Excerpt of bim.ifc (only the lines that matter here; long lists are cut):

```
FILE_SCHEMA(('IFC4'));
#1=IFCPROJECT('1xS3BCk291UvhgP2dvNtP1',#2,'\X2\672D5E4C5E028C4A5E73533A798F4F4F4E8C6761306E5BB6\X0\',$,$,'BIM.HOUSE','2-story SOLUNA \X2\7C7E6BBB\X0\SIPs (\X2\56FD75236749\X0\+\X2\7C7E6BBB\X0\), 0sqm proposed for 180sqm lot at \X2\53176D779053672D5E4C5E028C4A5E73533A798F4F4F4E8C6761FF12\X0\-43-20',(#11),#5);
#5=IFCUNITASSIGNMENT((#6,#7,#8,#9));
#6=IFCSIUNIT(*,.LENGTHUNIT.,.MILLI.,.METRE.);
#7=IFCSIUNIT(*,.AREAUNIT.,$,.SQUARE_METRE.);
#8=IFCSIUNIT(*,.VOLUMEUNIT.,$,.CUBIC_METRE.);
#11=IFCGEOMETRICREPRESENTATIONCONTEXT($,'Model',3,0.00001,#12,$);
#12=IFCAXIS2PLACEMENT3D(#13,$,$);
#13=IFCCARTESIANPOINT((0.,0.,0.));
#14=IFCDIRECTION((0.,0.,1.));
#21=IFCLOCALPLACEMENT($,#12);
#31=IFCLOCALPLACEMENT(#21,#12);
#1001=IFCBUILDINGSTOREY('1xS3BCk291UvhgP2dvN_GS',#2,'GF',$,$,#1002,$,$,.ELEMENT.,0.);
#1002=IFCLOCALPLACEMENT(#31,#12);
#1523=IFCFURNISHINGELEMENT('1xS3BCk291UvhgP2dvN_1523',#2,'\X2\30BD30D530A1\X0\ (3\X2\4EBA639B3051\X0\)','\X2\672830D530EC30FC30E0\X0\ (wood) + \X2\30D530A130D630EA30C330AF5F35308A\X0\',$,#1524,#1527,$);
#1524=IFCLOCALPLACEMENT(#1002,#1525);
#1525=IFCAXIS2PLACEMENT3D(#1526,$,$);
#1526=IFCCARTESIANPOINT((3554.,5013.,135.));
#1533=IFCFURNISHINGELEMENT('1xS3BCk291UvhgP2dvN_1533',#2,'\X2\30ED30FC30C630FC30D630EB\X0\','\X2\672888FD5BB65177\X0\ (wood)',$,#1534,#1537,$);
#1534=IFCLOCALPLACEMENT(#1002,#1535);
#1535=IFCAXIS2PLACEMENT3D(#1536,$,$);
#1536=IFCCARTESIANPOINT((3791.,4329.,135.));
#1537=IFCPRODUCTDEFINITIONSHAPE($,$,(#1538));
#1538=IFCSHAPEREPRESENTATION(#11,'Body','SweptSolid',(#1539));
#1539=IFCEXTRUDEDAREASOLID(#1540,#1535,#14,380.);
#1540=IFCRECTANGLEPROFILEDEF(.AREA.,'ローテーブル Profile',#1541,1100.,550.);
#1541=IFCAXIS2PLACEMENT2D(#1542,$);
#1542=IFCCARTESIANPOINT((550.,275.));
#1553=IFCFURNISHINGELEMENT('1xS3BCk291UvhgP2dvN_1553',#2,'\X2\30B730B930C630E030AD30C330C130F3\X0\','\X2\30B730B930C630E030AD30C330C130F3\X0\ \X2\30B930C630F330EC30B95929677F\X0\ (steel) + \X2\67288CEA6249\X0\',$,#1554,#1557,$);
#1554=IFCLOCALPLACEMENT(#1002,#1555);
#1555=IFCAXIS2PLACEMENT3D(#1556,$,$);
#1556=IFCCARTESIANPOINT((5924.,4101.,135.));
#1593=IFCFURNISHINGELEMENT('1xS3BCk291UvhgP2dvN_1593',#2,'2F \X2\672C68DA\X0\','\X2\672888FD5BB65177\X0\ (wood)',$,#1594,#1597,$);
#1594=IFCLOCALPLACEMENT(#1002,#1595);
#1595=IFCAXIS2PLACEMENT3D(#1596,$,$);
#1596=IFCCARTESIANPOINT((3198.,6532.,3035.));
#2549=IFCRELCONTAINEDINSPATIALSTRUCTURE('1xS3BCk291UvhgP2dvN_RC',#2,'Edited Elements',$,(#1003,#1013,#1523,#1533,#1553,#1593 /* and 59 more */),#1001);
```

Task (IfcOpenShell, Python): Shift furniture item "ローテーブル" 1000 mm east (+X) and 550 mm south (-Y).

```python
import ifcopenshell
import ifcopenshell.api.geometry
import ifcopenshell.util.placement

model = ifcopenshell.open("bim.ifc")

item = model.by_id(1533)
matrix = ifcopenshell.util.placement.get_local_placement(item.ObjectPlacement)
matrix[0, 3] += 1000.0
matrix[1, 3] -= 550.0
ifcopenshell.api.geometry.edit_object_placement(model, product=item, matrix=matrix, is_si=False)

print(ifcopenshell.util.placement.get_local_placement(item.ObjectPlacement).round(3) + 0.0)

model.write("bim_v2.ifc")
```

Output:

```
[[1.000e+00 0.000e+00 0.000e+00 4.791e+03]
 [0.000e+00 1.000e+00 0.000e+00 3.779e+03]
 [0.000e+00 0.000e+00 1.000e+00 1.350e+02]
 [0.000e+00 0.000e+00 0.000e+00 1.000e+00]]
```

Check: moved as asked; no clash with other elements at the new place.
